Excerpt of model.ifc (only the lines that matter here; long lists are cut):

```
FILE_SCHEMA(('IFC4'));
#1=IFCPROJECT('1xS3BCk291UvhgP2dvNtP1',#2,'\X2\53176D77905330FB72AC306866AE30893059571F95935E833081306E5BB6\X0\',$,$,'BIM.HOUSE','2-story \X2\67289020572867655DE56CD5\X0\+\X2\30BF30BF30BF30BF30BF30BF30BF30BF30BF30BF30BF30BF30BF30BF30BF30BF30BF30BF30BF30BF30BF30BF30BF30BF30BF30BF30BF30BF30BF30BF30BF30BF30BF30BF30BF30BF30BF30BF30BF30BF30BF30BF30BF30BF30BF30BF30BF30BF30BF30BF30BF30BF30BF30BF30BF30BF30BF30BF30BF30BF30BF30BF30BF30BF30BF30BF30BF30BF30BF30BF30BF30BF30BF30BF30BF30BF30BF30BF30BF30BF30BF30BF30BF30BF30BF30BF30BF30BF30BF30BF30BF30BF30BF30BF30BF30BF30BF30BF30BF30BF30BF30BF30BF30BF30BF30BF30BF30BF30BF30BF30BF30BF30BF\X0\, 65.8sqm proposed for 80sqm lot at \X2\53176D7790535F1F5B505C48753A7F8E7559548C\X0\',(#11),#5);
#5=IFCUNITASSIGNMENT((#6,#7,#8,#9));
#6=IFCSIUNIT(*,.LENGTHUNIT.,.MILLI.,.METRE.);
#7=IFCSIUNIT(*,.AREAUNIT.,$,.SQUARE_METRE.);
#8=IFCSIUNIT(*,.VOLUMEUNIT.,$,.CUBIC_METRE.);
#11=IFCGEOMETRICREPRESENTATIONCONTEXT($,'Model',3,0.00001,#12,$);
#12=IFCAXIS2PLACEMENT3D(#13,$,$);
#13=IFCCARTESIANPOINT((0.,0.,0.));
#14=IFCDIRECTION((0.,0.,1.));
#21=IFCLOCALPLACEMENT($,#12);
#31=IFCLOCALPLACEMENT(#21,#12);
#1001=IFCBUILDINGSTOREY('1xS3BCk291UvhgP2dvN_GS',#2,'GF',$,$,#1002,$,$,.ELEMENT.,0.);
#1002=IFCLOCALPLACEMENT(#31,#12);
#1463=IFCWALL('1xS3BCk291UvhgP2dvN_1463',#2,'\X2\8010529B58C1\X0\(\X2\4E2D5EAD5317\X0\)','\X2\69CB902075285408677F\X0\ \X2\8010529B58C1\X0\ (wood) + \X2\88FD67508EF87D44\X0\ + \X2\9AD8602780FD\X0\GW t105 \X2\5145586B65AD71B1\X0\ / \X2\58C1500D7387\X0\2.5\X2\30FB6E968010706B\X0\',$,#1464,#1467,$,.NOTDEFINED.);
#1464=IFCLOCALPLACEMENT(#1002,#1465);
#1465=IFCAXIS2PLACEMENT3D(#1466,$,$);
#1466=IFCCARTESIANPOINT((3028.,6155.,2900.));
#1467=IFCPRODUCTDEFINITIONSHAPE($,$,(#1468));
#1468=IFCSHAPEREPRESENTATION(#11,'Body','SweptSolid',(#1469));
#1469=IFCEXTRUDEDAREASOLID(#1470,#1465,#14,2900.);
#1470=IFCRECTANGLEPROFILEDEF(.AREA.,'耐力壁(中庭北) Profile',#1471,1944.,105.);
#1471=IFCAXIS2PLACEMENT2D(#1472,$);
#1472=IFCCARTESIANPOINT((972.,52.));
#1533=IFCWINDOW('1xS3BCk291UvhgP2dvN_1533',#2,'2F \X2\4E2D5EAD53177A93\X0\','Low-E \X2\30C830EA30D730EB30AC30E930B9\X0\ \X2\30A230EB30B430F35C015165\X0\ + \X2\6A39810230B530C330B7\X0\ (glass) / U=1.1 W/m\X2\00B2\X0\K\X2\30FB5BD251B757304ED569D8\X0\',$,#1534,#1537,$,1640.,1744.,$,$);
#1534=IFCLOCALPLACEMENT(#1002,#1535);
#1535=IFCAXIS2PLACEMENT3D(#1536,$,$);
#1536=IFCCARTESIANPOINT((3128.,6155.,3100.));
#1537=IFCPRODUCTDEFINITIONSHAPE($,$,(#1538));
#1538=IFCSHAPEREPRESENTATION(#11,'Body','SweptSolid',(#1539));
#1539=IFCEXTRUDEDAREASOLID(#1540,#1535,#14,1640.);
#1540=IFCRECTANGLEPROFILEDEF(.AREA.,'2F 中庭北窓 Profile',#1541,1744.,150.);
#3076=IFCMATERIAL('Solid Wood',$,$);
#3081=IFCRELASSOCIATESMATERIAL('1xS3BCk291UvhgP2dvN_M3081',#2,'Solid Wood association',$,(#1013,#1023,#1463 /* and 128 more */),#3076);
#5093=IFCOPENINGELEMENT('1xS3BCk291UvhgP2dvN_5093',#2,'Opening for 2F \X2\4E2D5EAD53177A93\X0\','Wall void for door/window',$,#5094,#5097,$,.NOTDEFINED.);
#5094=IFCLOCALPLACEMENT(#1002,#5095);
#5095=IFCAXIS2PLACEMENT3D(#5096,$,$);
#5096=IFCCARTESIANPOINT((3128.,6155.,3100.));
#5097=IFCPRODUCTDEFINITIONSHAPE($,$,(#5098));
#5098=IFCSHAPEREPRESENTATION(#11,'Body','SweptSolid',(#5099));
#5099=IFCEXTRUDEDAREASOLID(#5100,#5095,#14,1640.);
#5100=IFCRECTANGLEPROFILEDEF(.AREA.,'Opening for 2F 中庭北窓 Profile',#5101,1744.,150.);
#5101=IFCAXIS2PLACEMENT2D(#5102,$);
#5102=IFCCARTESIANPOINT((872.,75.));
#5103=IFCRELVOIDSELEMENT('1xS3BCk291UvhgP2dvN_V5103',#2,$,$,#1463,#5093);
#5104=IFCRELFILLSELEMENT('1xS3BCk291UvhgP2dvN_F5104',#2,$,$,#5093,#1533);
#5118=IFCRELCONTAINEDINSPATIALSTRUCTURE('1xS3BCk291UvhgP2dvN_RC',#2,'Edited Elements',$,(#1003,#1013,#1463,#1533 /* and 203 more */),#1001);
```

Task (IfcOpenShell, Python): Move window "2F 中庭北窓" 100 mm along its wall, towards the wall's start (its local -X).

```python
import ifcopenshell
import ifcopenshell.api.geometry
import ifcopenshell.util.placement
import ifcopenshell.util.unit

model = ifcopenshell.open("model.ifc")
unit_scale = ifcopenshell.util.unit.calculate_unit_scale(model)

window = model.by_id(1533)
opening = window.FillsVoids[0].RelatingOpeningElement
wall = opening.VoidsElements[0].RelatingBuildingElement

wall_matrix = ifcopenshell.util.placement.get_local_placement(wall.ObjectPlacement)
shift = wall_matrix[:3, 0] * -0.1 / unit_scale
before = ifcopenshell.util.placement.get_local_placement(window.ObjectPlacement)[:3, 3].copy()

# The window is not placed relative to its opening, so move both.
for product in (opening, window):
    matrix = ifcopenshell.util.placement.get_local_placement(product.ObjectPlacement)
    matrix[:3, 3] += shift
    ifcopenshell.api.geometry.edit_object_placement(model, product=product, matrix=matrix, is_si=False)

after = ifcopenshell.util.placement.get_local_placement(window.ObjectPlacement)[:3, 3]
print("window moved by", (after - before).round(3) + 0.0)

model.write("model_rev.ifc")
```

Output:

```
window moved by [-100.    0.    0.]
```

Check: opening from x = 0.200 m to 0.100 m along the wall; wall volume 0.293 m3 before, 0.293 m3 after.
